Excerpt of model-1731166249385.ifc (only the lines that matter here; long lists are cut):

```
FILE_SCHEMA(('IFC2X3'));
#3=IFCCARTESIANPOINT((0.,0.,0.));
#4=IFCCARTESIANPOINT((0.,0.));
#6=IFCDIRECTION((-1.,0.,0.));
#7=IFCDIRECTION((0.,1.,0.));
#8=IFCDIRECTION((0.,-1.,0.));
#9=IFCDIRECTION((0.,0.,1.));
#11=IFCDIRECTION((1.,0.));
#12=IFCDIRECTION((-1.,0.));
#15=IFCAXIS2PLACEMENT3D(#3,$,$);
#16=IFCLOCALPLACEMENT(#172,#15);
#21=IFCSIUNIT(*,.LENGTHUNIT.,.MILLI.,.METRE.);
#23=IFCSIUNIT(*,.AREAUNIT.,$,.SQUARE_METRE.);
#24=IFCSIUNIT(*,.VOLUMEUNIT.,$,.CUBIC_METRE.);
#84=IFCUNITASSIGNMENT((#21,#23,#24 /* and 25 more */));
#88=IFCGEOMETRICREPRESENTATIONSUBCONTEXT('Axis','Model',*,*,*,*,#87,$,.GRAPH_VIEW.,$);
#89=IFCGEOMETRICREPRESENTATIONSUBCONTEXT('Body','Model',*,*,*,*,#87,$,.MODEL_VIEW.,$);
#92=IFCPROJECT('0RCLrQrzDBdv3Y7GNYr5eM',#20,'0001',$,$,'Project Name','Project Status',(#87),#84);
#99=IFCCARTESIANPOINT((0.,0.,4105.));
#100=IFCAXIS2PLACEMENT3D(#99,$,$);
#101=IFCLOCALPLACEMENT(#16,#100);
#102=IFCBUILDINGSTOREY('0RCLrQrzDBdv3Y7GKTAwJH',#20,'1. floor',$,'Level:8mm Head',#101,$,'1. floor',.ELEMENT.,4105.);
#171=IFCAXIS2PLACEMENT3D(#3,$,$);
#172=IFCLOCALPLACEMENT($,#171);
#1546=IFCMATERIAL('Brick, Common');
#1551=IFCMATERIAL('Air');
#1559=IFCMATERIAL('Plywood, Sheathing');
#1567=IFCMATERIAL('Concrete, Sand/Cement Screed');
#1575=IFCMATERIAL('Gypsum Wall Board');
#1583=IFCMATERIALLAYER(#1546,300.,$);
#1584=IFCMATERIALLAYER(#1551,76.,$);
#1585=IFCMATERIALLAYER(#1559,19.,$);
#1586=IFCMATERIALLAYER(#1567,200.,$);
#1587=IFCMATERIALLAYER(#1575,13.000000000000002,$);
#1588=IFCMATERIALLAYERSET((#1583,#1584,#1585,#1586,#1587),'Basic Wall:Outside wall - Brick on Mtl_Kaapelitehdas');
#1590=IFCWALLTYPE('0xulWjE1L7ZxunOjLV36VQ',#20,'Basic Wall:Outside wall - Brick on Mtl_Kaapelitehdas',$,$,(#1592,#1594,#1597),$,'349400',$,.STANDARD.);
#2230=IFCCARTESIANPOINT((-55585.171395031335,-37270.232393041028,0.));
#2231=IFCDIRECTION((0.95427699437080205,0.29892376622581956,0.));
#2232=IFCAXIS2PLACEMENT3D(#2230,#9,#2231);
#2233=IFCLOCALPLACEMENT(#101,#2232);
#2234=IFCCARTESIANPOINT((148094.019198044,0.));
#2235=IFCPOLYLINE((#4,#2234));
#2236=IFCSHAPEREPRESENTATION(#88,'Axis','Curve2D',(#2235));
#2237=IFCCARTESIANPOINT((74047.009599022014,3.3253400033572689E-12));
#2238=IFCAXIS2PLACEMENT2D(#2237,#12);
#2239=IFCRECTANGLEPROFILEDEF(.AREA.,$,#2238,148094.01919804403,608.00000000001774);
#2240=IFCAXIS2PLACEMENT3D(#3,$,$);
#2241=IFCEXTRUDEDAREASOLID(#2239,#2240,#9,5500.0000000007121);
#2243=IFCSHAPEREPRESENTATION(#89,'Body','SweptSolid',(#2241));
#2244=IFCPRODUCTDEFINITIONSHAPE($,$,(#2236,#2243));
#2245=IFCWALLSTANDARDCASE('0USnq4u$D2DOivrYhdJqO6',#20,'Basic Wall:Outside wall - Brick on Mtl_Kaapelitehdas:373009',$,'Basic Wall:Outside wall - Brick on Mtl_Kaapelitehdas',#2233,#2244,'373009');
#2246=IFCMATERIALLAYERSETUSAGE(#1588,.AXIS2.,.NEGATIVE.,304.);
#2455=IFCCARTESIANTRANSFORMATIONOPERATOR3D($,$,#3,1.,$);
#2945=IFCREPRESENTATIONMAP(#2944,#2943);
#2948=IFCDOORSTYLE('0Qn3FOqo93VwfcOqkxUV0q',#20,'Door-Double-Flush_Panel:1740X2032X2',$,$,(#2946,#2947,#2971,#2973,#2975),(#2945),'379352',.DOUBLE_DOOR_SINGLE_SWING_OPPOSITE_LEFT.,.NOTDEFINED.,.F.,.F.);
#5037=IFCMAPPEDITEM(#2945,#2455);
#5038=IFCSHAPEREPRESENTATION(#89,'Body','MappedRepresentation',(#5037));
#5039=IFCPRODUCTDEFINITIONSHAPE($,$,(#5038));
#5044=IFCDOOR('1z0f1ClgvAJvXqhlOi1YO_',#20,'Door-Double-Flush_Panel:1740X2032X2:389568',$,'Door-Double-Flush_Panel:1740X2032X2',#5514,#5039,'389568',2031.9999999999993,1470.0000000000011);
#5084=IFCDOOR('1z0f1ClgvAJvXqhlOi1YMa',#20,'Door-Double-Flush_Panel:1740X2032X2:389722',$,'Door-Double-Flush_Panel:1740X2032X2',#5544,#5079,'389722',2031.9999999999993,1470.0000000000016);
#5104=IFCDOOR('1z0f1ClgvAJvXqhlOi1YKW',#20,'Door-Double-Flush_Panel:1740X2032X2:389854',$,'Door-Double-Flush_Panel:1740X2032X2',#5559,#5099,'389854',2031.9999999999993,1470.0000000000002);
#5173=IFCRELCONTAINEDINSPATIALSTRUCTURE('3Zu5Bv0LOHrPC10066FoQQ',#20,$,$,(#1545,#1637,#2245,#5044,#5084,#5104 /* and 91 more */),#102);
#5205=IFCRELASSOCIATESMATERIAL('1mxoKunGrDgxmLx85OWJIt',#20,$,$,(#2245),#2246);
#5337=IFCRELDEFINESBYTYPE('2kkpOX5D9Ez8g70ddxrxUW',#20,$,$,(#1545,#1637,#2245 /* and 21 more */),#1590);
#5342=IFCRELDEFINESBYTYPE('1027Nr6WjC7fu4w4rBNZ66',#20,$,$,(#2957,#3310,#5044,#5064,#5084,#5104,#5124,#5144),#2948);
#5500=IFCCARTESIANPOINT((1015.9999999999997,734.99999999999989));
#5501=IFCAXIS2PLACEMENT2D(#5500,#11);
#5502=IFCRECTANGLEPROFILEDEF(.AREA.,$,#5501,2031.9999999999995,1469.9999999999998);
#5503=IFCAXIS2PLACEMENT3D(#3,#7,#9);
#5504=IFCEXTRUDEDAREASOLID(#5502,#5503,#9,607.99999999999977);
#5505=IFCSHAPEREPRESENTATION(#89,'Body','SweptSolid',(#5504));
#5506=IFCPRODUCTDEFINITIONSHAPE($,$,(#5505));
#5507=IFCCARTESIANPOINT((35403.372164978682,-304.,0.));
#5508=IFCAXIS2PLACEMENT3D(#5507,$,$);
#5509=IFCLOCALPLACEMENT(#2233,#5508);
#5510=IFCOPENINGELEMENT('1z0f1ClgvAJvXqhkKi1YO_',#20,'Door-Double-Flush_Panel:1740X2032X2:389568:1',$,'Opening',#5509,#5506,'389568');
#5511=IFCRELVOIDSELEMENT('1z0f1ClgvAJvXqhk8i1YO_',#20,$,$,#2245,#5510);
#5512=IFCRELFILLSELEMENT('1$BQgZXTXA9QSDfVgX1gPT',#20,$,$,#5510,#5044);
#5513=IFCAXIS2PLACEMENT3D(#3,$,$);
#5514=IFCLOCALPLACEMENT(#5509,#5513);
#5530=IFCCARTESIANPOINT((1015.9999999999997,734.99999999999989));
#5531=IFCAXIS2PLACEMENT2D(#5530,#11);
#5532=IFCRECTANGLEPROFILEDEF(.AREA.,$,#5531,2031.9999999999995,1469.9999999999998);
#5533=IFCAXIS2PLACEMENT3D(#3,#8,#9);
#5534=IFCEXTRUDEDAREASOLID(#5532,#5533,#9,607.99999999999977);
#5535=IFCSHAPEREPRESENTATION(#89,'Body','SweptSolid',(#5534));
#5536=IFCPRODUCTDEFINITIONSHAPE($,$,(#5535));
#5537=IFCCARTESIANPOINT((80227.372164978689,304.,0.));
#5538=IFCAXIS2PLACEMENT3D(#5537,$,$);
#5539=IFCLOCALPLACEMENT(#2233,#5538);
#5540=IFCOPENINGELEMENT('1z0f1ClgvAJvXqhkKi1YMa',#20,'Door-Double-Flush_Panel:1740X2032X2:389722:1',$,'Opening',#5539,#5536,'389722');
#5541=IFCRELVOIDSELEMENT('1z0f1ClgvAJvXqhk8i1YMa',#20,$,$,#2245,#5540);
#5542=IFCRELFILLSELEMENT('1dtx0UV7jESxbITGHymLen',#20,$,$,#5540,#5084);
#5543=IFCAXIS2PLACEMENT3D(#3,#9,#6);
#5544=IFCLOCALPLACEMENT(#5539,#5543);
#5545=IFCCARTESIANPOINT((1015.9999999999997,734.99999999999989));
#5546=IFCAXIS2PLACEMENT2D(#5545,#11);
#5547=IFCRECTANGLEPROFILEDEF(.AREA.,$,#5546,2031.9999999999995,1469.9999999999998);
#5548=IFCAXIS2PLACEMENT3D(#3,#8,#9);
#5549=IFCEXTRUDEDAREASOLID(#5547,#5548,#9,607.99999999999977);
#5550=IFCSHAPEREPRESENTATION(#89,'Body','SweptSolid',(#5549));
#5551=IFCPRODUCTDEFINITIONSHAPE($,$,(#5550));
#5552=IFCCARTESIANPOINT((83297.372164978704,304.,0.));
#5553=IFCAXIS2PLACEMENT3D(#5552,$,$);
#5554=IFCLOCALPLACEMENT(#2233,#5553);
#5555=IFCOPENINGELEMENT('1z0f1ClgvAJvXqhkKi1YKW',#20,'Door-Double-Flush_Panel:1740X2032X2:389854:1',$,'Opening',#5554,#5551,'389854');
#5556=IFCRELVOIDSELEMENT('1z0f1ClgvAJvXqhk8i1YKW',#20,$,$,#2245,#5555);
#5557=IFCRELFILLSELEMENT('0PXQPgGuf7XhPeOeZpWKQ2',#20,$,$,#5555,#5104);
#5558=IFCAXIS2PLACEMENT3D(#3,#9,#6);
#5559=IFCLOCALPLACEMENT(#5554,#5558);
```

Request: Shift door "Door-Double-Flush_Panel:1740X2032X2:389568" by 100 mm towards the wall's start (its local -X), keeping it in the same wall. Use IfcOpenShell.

```python
import ifcopenshell
import ifcopenshell.api.geometry
import ifcopenshell.util.placement

model = ifcopenshell.open("model-1731166249385.ifc")

door = model.by_guid("1z0f1ClgvAJvXqhlOi1YO_")
opening = door.FillsVoids[0].RelatingOpeningElement
wall = opening.VoidsElements[0].RelatingBuildingElement

wall_matrix = ifcopenshell.util.placement.get_local_placement(wall.ObjectPlacement)
shift = wall_matrix[:3, 0] * -100.0
before = ifcopenshell.util.placement.get_local_placement(door.ObjectPlacement)[:3, 3].copy()

# The door is placed relative to its opening, so it follows when the opening moves.
matrix = ifcopenshell.util.placement.get_local_placement(opening.ObjectPlacement)
matrix[:3, 3] += shift
ifcopenshell.api.geometry.edit_object_placement(
    model, product=opening, matrix=matrix, is_si=False, should_transform_children=True
)

after = ifcopenshell.util.placement.get_local_placement(door.ObjectPlacement)[:3, 3]
print("door moved by", (after - before).round(3) + 0.0)

model.write("model-1731166249385_edited.ifc")
```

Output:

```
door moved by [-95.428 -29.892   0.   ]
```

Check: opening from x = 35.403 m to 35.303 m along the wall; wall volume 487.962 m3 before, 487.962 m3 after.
